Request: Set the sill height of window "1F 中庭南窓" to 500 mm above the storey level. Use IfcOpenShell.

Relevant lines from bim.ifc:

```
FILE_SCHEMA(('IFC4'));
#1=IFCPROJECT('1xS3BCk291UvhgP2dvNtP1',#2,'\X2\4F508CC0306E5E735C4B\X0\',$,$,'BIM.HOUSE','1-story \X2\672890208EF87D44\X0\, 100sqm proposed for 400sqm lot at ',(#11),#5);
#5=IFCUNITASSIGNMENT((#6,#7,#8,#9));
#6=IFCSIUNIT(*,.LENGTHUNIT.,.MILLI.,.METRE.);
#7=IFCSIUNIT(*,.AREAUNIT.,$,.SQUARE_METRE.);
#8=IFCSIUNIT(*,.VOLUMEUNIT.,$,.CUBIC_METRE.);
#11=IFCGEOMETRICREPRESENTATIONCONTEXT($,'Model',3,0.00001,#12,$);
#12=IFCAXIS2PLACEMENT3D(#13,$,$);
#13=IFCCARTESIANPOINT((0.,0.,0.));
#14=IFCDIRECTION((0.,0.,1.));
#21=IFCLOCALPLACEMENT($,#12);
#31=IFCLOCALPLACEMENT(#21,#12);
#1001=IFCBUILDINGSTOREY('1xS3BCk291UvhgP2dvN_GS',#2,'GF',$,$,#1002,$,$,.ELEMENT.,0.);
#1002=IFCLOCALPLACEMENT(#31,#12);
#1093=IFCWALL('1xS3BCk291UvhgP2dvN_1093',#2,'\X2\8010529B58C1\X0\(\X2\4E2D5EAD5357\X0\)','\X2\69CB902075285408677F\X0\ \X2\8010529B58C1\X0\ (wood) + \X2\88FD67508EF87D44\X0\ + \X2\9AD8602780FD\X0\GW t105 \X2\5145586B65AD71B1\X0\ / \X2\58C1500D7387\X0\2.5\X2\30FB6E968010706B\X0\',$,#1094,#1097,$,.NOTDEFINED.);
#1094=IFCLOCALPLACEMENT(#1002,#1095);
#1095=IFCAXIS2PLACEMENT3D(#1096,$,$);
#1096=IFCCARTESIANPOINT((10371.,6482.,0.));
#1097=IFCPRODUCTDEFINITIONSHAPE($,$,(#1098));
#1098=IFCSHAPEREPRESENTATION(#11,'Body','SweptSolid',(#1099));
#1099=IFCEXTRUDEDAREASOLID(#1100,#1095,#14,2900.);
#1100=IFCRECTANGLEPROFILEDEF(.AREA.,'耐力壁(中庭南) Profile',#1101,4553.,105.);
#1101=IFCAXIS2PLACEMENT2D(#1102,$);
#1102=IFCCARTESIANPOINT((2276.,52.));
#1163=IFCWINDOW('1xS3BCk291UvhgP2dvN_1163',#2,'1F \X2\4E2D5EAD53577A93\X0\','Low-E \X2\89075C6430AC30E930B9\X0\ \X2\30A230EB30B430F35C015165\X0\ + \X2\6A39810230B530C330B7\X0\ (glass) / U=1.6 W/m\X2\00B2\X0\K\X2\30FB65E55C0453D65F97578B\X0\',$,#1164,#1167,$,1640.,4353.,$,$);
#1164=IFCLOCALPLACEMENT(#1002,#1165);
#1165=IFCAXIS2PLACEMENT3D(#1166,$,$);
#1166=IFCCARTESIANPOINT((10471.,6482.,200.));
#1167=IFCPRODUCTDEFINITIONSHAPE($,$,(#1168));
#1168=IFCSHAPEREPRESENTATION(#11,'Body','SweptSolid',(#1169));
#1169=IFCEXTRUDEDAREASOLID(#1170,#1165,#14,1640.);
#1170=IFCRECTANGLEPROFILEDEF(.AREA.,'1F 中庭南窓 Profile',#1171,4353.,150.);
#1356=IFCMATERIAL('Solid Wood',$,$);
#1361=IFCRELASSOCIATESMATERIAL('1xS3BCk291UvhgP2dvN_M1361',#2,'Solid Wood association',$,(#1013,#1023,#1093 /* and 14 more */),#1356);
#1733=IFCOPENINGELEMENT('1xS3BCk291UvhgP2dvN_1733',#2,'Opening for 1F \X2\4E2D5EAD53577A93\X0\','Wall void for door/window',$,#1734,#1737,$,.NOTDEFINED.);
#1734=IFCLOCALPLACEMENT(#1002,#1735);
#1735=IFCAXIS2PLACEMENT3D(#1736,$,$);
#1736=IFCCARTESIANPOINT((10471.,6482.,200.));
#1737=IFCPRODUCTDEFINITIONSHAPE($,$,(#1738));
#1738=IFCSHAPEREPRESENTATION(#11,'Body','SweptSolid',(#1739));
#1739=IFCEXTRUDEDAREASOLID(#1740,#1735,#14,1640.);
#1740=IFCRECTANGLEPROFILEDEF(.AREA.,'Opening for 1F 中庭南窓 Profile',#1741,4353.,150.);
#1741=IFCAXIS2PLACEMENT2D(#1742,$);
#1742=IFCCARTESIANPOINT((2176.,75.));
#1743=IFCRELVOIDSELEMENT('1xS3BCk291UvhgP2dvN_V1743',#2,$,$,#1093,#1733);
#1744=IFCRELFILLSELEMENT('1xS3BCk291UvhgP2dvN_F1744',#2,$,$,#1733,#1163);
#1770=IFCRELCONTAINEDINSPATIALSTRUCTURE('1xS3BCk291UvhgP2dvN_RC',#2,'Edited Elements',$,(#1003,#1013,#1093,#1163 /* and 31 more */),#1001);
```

```python
import numpy as np
import ifcopenshell
import ifcopenshell.api.geometry
import ifcopenshell.geom
import ifcopenshell.util.element
import ifcopenshell.util.placement
import ifcopenshell.util.shape
import ifcopenshell.util.unit

model = ifcopenshell.open("bim.ifc")
unit_scale = ifcopenshell.util.unit.calculate_unit_scale(model)

window = model.by_guid("1xS3BCk291UvhgP2dvN_1163")
opening = window.FillsVoids[0].RelatingOpeningElement
storey = ifcopenshell.util.element.get_container(window, ifc_class="IfcBuildingStorey")
level = ifcopenshell.util.placement.get_local_placement(storey.ObjectPlacement)[2, 3]

# The opening's origin need not be at the sill, so measure its lowest point.
shape = ifcopenshell.geom.create_shape(ifcopenshell.geom.settings(), opening)
bottom = ifcopenshell.util.shape.get_shape_bottom_elevation(shape, shape.geometry) / unit_scale
dz = level + 0.5 / unit_scale - bottom

shift = np.array([0.0, 0.0, dz])
# The window is not placed relative to its opening, so move both.
for product in (opening, window):
    matrix = ifcopenshell.util.placement.get_local_placement(product.ObjectPlacement)
    matrix[:3, 3] += shift
    ifcopenshell.api.geometry.edit_object_placement(model, product=product, matrix=matrix, is_si=False)

print(f"moved by {dz * unit_scale:+.3f} m")

model.write("bim-out.ifc")
```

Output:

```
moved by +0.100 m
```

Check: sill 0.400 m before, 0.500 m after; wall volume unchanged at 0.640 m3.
